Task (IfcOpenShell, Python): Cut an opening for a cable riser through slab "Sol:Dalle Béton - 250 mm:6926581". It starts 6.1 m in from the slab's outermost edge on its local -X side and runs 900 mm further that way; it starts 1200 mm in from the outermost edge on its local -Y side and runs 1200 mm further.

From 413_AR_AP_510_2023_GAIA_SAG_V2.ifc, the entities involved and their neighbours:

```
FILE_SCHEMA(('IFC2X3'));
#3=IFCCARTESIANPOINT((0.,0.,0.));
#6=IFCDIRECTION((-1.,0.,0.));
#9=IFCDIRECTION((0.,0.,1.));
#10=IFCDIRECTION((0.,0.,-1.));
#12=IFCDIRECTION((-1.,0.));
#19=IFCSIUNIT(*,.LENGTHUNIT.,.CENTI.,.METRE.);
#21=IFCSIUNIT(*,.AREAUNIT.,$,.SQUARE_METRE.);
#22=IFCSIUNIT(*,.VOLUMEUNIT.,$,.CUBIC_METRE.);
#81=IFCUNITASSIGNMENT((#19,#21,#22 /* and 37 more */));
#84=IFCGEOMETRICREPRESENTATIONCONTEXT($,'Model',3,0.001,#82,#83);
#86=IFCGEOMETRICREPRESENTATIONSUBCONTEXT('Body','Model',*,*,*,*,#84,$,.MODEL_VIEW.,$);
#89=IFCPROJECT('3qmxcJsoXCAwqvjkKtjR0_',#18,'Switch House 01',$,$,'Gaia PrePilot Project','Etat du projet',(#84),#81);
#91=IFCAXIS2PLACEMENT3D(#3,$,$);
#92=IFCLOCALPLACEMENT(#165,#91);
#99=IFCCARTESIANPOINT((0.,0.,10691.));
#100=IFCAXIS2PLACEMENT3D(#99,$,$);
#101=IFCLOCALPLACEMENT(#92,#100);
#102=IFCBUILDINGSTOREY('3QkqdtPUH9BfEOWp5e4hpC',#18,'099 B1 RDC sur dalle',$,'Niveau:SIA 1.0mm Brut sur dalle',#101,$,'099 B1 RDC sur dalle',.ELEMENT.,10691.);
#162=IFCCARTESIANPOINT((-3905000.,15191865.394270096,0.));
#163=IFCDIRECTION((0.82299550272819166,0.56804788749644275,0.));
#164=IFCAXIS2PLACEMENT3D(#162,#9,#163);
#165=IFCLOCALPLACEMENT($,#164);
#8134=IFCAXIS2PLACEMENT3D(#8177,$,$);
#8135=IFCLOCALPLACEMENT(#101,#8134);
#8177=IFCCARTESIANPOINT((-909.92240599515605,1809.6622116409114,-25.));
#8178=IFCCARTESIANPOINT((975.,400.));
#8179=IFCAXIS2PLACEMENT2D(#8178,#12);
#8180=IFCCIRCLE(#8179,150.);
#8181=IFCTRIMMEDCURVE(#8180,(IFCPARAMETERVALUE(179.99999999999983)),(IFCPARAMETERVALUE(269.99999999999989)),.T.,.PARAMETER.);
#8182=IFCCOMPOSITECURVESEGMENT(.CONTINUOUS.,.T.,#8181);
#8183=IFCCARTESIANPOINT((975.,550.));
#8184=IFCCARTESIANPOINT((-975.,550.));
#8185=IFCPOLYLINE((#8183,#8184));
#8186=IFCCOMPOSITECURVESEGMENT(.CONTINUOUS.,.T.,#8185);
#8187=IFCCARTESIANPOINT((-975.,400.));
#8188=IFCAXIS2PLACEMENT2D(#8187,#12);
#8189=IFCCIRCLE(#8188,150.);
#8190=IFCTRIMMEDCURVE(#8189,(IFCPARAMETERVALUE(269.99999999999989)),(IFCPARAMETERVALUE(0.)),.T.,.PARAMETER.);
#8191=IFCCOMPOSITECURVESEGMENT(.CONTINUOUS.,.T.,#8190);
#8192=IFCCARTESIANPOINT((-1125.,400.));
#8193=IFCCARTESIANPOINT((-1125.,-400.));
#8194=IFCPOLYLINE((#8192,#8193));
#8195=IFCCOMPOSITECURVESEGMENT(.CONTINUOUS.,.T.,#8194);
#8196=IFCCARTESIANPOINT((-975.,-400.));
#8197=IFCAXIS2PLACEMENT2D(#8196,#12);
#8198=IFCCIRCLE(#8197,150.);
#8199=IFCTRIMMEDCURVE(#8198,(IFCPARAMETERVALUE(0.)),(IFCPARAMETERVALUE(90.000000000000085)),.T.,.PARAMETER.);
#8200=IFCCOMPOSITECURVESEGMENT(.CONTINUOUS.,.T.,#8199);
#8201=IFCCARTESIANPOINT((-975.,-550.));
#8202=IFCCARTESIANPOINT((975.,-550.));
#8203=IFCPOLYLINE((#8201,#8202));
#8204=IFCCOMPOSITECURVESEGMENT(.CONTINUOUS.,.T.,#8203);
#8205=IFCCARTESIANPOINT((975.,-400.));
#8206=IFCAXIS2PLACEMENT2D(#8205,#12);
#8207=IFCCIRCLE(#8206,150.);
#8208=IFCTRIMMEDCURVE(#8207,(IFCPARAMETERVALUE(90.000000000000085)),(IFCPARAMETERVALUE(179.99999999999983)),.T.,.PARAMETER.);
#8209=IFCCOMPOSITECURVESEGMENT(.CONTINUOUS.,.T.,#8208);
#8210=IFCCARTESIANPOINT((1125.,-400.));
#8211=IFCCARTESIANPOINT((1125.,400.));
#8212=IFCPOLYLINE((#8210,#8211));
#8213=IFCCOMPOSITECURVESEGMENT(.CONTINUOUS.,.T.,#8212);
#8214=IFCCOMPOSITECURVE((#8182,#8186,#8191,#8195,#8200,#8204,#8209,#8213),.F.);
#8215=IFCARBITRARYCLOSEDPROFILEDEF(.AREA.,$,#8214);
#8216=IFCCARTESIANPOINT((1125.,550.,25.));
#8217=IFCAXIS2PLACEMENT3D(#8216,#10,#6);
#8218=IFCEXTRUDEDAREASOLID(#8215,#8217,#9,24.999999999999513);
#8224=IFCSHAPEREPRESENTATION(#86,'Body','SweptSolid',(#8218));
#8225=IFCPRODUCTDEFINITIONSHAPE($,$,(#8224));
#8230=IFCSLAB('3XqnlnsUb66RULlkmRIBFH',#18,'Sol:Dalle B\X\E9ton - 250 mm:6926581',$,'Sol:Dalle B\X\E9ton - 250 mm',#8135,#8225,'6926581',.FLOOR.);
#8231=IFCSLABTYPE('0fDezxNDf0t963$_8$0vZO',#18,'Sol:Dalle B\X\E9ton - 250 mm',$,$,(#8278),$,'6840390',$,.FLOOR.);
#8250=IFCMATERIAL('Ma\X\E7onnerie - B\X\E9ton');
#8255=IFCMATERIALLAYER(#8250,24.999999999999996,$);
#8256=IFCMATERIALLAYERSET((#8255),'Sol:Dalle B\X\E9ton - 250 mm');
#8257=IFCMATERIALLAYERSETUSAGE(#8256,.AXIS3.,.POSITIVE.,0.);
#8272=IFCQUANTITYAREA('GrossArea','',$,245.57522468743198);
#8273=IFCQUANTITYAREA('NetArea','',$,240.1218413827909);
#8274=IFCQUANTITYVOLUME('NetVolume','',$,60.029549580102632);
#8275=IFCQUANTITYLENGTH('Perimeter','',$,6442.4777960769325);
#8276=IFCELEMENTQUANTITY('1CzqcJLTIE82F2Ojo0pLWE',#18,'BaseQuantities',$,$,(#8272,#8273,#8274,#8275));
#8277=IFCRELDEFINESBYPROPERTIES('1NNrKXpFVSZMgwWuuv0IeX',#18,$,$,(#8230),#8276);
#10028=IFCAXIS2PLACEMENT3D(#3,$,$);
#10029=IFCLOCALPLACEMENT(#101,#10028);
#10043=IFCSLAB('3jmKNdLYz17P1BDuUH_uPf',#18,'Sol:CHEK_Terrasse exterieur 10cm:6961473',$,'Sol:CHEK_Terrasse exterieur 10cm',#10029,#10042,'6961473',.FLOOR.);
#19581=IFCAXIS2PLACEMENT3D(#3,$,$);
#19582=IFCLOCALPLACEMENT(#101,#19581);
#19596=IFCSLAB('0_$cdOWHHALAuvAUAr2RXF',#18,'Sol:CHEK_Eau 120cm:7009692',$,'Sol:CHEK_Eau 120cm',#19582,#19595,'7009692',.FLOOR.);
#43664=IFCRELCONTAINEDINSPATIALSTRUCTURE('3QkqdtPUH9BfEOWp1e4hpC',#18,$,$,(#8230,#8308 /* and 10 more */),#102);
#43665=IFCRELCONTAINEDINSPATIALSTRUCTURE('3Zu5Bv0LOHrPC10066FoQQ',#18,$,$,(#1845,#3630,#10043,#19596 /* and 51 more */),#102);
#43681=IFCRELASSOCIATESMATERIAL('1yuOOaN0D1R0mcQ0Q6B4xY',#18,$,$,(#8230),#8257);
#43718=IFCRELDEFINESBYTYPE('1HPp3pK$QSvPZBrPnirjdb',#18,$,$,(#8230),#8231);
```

```python
import numpy as np
import ifcopenshell
import ifcopenshell.api.feature
import ifcopenshell.api.geometry
import ifcopenshell.api.pset
import ifcopenshell.api.root
import ifcopenshell.geom
import ifcopenshell.util.element
import ifcopenshell.util.placement
import ifcopenshell.util.representation
import ifcopenshell.util.shape
import ifcopenshell.util.unit

model = ifcopenshell.open("413_AR_AP_510_2023_GAIA_SAG_V2.ifc")
unit_scale = ifcopenshell.util.unit.calculate_unit_scale(model)
area_scale = ifcopenshell.util.unit.calculate_unit_scale(model, "AREAUNIT")
volume_scale = ifcopenshell.util.unit.calculate_unit_scale(model, "VOLUMEUNIT")
settings = ifcopenshell.geom.settings()


def volume(element):
    """Net volume in cubic metres, openings subtracted."""
    shape = ifcopenshell.geom.create_shape(settings, element)
    return ifcopenshell.util.shape.get_volume(shape.geometry)


slab = model.by_guid("3XqnlnsUb66RULlkmRIBFH")
before = volume(slab)

# Extent in the slab's own axes, in metres. The edges named are its -X and -Y sides.
slab_shape = ifcopenshell.geom.create_shape(settings, slab)
vertices = ifcopenshell.util.shape.get_vertices(slab_shape.geometry)
x_min, y_min, bottom = vertices.min(axis=0)
top = vertices[:, 2].max()

opening = ifcopenshell.api.root.create_entity(model, ifc_class="IfcOpeningElement", name="Cable riser opening")
context = ifcopenshell.util.representation.get_context(model, "Model", "Body", "MODEL_VIEW")
width, depth = 0.9, 1.2
outline = [(0.0, 0.0), (width, 0.0), (width, depth), (0.0, depth), (0.0, 0.0)]
# Overshoot both faces by 50 mm so the cut is clean.
shape = ifcopenshell.api.geometry.add_slab_representation(
    model, context=context, depth=top - bottom + 0.1, polyline=outline
)
ifcopenshell.api.geometry.assign_representation(model, product=opening, representation=shape)

matrix = ifcopenshell.util.placement.get_local_placement(slab.ObjectPlacement)
matrix[:, 3] = matrix @ np.append(np.array([x_min + 6.1, y_min + 1.2, bottom - 0.05]) / unit_scale, 1.0)
ifcopenshell.api.geometry.edit_object_placement(model, product=opening, matrix=matrix, is_si=False)
ifcopenshell.api.feature.add_feature(model, feature=opening, element=slab)

after = volume(slab)

# Update the slab's stored quantities.
qto = model.by_id(ifcopenshell.util.element.get_pset(slab, "BaseQuantities", should_inherit=False)["id"])
ifcopenshell.api.pset.edit_qto(model, qto=qto, properties={
    "NetArea": after / (top - bottom) / area_scale,
    "NetVolume": after / volume_scale,
})

print(f"slab volume {before:.3f} -> {after:.3f} m3")

model.write("413_AR_AP_510_2023_GAIA_SAG_V2_updated.ifc")
```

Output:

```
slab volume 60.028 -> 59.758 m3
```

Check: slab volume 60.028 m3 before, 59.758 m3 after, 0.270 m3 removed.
